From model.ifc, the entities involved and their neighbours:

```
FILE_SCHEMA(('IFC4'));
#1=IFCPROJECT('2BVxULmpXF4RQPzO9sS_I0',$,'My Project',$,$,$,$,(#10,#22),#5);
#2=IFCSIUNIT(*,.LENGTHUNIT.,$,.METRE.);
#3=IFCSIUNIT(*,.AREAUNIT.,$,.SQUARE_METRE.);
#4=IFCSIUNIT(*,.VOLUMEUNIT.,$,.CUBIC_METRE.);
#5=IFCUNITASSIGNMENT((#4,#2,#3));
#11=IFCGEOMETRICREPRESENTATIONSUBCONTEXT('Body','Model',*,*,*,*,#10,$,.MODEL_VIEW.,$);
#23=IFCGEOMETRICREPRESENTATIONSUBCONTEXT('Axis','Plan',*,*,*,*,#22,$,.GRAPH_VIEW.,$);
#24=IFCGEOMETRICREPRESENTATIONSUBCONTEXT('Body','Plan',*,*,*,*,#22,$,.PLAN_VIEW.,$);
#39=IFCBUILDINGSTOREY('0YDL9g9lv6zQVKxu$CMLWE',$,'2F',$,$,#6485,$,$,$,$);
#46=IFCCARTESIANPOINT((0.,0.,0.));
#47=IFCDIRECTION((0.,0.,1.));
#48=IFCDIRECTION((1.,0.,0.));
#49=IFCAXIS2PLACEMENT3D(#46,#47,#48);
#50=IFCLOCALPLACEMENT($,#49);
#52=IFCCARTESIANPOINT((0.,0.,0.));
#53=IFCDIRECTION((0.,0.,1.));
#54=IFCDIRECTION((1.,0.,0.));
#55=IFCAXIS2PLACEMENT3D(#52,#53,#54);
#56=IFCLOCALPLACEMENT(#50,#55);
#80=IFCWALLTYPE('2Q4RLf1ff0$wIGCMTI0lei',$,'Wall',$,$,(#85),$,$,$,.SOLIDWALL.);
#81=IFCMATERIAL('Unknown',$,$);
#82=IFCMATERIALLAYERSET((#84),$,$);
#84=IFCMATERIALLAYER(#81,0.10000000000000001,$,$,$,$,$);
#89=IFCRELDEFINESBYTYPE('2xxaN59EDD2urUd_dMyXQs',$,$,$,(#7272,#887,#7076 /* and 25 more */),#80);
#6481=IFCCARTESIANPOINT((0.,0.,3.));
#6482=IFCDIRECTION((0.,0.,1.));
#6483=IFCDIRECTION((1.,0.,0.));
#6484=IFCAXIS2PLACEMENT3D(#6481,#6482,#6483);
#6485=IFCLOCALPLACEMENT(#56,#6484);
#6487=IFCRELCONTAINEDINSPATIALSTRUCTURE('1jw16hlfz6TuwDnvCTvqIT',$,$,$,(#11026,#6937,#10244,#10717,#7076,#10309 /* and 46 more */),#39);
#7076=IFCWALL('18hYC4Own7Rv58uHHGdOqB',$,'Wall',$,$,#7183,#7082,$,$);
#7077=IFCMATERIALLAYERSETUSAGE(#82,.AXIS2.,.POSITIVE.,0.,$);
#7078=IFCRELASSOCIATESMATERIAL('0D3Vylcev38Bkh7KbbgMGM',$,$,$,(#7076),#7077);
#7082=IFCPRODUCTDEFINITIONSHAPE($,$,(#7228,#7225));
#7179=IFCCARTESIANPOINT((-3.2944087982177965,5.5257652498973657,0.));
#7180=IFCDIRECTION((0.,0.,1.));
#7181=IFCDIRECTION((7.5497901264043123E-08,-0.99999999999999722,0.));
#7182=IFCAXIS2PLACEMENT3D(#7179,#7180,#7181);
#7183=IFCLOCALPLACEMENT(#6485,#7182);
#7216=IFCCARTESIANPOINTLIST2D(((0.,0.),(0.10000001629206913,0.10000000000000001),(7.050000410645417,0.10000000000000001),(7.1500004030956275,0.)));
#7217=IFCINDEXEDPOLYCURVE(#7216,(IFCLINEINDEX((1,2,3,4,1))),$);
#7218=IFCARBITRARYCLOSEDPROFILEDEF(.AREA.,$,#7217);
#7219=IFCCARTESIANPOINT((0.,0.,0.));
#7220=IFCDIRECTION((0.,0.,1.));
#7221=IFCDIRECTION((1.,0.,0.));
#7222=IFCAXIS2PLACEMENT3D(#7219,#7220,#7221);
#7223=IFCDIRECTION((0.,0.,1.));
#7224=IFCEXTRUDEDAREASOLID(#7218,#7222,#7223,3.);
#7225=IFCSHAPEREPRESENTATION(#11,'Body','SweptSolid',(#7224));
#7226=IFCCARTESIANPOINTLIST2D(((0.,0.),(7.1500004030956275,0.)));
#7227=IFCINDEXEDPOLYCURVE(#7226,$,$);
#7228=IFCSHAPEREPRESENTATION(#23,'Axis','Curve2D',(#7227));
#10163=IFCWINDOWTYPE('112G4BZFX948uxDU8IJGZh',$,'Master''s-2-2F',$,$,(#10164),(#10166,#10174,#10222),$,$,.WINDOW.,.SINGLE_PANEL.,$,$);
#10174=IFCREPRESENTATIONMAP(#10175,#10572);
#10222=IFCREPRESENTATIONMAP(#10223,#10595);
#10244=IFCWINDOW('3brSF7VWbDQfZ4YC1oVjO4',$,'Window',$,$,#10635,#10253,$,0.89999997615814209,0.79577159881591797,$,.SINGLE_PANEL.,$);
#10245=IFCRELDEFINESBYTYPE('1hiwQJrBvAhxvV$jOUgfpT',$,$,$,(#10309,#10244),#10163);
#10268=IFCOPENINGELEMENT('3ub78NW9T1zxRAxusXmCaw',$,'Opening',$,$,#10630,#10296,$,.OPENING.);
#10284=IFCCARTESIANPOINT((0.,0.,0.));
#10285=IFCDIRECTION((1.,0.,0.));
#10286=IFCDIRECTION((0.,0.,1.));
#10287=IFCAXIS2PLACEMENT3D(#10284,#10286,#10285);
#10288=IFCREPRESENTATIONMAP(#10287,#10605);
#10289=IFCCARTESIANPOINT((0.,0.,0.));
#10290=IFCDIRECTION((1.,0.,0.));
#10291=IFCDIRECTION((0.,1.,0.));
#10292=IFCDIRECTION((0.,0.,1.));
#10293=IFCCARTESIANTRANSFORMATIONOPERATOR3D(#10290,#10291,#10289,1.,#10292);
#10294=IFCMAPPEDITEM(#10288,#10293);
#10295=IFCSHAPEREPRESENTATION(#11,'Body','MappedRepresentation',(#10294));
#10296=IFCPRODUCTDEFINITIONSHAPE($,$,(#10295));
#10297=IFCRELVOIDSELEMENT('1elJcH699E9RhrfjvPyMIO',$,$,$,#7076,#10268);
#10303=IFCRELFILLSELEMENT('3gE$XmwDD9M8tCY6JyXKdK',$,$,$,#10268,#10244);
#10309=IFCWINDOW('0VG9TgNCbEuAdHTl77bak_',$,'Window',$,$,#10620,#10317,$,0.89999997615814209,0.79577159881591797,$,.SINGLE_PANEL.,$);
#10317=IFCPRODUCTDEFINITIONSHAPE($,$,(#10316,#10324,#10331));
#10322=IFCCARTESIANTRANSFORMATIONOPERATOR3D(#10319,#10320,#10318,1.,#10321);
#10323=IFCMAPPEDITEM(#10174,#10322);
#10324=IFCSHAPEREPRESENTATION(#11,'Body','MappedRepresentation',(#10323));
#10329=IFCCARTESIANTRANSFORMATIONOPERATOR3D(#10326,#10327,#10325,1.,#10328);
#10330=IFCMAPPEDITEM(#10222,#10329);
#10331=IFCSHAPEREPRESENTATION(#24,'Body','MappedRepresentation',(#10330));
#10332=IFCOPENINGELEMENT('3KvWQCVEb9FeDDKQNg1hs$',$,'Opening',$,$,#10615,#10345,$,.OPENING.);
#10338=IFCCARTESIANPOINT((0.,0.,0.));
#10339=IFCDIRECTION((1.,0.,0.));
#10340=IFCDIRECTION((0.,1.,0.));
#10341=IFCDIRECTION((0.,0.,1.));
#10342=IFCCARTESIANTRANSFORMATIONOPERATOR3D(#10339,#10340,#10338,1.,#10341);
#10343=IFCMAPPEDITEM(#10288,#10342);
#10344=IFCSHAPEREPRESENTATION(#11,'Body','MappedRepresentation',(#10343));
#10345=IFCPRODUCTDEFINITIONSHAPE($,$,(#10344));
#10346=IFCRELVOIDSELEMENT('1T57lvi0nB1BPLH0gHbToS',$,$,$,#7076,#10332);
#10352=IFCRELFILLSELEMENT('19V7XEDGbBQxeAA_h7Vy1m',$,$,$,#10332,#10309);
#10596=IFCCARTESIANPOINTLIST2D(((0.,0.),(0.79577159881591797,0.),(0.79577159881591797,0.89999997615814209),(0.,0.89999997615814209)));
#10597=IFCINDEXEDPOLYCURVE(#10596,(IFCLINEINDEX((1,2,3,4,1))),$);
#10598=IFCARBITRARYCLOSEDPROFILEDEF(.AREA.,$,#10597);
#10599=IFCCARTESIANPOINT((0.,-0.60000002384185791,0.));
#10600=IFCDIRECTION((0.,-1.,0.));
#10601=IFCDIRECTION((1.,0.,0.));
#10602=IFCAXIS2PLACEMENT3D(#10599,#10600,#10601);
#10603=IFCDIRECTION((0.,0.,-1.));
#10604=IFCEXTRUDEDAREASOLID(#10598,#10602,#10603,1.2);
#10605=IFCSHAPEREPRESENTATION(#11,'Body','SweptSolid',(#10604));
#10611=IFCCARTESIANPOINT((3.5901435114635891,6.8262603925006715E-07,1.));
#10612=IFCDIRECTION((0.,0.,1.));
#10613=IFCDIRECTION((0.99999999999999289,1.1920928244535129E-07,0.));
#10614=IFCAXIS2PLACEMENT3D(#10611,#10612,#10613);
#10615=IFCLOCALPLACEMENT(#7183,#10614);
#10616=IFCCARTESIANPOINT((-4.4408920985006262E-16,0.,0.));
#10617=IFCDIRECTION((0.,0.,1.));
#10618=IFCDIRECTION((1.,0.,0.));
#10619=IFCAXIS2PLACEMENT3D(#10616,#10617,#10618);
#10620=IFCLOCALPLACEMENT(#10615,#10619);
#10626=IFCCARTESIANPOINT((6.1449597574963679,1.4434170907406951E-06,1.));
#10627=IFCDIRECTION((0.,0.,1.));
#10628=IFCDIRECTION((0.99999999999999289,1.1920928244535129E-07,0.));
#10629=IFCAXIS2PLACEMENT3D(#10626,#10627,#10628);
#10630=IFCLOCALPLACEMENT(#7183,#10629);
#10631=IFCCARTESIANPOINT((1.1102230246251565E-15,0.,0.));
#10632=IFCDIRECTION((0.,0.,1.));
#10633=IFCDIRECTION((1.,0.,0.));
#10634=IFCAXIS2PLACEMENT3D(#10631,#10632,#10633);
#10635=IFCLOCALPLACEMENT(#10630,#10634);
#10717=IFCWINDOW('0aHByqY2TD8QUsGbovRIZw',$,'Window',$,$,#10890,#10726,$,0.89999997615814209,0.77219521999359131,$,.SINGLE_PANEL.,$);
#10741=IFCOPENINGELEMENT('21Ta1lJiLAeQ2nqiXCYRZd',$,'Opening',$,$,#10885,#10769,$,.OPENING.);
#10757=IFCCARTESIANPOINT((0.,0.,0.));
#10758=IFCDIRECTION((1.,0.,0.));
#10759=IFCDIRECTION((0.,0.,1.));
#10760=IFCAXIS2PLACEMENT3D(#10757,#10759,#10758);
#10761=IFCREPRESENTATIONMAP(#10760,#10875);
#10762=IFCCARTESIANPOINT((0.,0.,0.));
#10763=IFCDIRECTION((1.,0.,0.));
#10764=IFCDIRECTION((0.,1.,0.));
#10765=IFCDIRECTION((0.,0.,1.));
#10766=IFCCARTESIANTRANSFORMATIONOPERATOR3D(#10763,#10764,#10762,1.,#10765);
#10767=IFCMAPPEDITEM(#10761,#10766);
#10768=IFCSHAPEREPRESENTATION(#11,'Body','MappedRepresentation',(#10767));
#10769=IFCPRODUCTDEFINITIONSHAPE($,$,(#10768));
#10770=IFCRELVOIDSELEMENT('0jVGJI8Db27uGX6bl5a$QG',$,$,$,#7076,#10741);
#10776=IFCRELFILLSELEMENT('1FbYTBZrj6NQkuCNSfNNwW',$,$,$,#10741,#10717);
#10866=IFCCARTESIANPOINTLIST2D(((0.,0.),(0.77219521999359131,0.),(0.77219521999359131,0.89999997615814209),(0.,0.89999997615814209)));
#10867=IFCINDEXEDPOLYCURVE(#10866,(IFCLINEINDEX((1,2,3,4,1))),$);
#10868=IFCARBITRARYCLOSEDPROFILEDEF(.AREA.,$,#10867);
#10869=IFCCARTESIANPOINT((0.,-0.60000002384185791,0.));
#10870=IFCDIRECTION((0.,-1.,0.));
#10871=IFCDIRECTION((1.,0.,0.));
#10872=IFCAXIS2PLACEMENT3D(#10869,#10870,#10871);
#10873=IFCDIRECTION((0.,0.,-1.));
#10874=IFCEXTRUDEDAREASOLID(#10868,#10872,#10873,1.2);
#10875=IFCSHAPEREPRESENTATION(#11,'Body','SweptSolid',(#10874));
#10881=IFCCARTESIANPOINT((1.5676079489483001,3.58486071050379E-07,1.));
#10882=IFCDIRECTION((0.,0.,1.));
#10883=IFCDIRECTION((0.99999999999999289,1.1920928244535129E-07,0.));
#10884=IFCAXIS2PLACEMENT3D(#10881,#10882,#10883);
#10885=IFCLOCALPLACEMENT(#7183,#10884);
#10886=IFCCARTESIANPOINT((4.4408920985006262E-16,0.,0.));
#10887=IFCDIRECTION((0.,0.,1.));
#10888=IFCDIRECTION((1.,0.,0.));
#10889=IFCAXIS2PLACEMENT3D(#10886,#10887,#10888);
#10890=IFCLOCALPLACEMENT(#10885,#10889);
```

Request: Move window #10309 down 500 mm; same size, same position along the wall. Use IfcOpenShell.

```python
import numpy as np
import ifcopenshell
import ifcopenshell.api.geometry
import ifcopenshell.util.placement
import ifcopenshell.util.unit

model = ifcopenshell.open("model.ifc")
unit_scale = ifcopenshell.util.unit.calculate_unit_scale(model)

window = model.by_id(10309)
opening = window.FillsVoids[0].RelatingOpeningElement
dz = -0.5

shift = np.array([0.0, 0.0, dz])
# The window is placed relative to its opening, so it follows when the opening moves.
matrix = ifcopenshell.util.placement.get_local_placement(opening.ObjectPlacement)
matrix[:3, 3] += shift
ifcopenshell.api.geometry.edit_object_placement(
    model, product=opening, matrix=matrix, is_si=False, should_transform_children=True
)

print(f"moved by {dz * unit_scale:+.3f} m")

model.write("model-out.ifc")
```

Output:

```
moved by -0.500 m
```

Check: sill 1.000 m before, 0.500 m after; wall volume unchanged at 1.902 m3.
